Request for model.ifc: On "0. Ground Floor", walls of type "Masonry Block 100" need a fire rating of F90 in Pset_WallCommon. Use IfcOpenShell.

First a look at what the model holds.

```python
import ifcopenshell
import ifcopenshell.util.element

model = ifcopenshell.open("model.ifc")
print(model.schema)
storey = next(s for s in model.by_type("IfcBuildingStorey") if s.Name == "0. Ground Floor")
walls = [e for e in ifcopenshell.util.element.get_decomposition(storey) if e.is_a("IfcWall")]
seen = {}
for e in walls:
    element_type = ifcopenshell.util.element.get_type(e)
    key = (element_type.Name if element_type != e and element_type else None, ifcopenshell.util.element.get_pset(e, "Pset_WallCommon", "FireRating"))
    seen[key] = seen.get(key, 0) + 1
for (name, value), count in sorted(seen.items(), key=str):
    print(count, "x", name, "|", value)
```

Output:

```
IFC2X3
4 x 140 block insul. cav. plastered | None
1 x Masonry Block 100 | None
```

```python
import ifcopenshell
import ifcopenshell.api.pset
import ifcopenshell.util.element

model = ifcopenshell.open("model.ifc")

storey = next(s for s in model.by_type("IfcBuildingStorey") if s.Name == "0. Ground Floor")
walls = [e for e in ifcopenshell.util.element.get_decomposition(storey) if e.is_a("IfcWall")]

count = 0
for e in walls:
    element_type = ifcopenshell.util.element.get_type(e)
    if element_type in (None, e) or element_type.Name != "Masonry Block 100":
        continue
    # add_pset returns the element's existing set when there is one.
    pset = ifcopenshell.api.pset.add_pset(model, product=e, name="Pset_WallCommon")
    ifcopenshell.api.pset.edit_pset(model, pset=pset, properties={"FireRating": "F90"})
    count += 1

print(count, "walls updated")

model.write("model_rev.ifc")
```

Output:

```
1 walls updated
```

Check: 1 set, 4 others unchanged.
